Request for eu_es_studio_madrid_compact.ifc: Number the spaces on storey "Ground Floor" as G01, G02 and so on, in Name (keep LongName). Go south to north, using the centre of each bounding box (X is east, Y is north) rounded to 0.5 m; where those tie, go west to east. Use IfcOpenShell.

First a look at what the model holds.

```python
import ifcopenshell
import ifcopenshell.util.element
import ifcopenshell.util.placement

model = ifcopenshell.open("eu_es_studio_madrid_compact.ifc")
print(model.schema)
storey = next(s for s in model.by_type("IfcBuildingStorey") if s.Name == "Ground Floor")
spaces = [e for e in ifcopenshell.util.element.get_decomposition(storey) if e.is_a("IfcSpace")]
for e in sorted(spaces, key=lambda e: e.id()):
    origin = ifcopenshell.util.placement.get_local_placement(e.ObjectPlacement)[:3, 3]
    print(e.id(), e.Name, e.LongName, origin.round(2) + 0.0, sep=" | ")
```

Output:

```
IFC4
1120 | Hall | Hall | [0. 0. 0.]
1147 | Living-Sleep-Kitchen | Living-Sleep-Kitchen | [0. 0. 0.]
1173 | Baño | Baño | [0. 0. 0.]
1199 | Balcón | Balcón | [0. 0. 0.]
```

```python
import ifcopenshell
import ifcopenshell.geom
import ifcopenshell.util.element
import ifcopenshell.util.shape

model = ifcopenshell.open("eu_es_studio_madrid_compact.ifc")
settings = ifcopenshell.geom.settings()
settings.set("use-world-coords", True)


def centre(element):
    shape = ifcopenshell.geom.create_shape(settings, element)
    return ifcopenshell.util.shape.get_bbox_centroid(shape.geometry)


storey = next(s for s in model.by_type("IfcBuildingStorey") if s.Name == "Ground Floor")
spaces = [e for e in ifcopenshell.util.element.get_decomposition(storey) if e.is_a("IfcSpace")]

# Insertion points can sit at a corner or the storey origin, so sort by the geometry (in metres).
centres = {e: centre(e) for e in spaces}
spaces.sort(key=lambda e: (round(centres[e][1] / 0.5), centres[e][0]))

for i, e in enumerate(spaces, start=1):
    number = f"G{i:02d}"
    e.Name = number
    print(e.id(), number)

model.write("eu_es_studio_madrid_compact_rev.ifc")
```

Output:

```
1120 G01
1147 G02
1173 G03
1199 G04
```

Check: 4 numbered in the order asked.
